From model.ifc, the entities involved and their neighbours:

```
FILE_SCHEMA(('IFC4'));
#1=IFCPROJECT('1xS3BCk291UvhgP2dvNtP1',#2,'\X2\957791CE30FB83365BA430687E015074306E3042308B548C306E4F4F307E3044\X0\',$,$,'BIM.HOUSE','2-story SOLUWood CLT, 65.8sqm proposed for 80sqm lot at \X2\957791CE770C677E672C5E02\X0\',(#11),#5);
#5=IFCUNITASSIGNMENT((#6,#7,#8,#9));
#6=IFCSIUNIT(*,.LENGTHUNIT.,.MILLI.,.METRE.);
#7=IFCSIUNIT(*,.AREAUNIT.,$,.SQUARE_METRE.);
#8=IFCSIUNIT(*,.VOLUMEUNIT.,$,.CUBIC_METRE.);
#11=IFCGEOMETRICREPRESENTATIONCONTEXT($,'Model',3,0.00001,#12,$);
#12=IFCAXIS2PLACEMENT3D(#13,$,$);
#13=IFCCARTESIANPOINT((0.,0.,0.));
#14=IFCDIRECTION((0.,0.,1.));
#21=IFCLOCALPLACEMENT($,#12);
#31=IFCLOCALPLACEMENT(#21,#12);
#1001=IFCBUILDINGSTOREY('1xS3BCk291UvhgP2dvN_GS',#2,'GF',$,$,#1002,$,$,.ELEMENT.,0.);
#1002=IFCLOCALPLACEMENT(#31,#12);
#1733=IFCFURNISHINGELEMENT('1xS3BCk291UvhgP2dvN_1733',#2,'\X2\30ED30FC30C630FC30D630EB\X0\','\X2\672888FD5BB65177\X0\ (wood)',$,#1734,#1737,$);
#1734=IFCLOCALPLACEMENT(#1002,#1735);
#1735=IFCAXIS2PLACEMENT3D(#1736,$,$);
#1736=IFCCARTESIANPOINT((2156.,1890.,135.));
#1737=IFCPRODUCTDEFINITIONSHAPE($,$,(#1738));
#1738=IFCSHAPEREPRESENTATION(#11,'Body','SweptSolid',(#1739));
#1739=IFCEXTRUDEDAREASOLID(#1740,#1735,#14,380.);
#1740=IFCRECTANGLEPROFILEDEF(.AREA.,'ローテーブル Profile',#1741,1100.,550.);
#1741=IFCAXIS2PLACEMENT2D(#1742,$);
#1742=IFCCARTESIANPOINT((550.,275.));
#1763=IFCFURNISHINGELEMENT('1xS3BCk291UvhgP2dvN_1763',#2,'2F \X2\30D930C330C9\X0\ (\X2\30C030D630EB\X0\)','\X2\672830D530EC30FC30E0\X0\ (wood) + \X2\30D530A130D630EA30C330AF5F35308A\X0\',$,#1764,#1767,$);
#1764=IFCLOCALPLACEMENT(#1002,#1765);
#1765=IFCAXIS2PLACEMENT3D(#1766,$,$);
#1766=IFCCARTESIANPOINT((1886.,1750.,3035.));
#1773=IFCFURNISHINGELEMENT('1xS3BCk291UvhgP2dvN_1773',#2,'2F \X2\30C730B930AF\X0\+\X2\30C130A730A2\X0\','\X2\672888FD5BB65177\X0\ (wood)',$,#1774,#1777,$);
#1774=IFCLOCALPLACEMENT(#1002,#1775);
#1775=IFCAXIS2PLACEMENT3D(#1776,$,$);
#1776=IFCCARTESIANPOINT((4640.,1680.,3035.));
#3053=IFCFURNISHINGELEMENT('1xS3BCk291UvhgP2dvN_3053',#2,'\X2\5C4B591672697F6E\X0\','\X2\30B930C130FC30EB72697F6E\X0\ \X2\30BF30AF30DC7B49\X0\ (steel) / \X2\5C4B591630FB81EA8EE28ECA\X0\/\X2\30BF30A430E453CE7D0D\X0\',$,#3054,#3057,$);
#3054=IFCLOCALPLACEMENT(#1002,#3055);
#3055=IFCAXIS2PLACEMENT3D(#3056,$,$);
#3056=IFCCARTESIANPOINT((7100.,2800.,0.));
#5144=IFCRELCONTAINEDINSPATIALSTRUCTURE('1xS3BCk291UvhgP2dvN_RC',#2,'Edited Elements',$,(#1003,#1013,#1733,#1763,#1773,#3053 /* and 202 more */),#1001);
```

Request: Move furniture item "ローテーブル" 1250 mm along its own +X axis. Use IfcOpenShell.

```python
import ifcopenshell
import ifcopenshell.api.geometry
import ifcopenshell.util.placement
import ifcopenshell.util.unit

model = ifcopenshell.open("model.ifc")
unit_scale = ifcopenshell.util.unit.calculate_unit_scale(model)

item = model.by_id(1733)
matrix = ifcopenshell.util.placement.get_local_placement(item.ObjectPlacement)
matrix[:3, 3] += matrix[:3, 0] * 1.25 / unit_scale
ifcopenshell.api.geometry.edit_object_placement(model, product=item, matrix=matrix, is_si=False)

print(ifcopenshell.util.placement.get_local_placement(item.ObjectPlacement).round(3) + 0.0)

model.write("model_v2.ifc")
```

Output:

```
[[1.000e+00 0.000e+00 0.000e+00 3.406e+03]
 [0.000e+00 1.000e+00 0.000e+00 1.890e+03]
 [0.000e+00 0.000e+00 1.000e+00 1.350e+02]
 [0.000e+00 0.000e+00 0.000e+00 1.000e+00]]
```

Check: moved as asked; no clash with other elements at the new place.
